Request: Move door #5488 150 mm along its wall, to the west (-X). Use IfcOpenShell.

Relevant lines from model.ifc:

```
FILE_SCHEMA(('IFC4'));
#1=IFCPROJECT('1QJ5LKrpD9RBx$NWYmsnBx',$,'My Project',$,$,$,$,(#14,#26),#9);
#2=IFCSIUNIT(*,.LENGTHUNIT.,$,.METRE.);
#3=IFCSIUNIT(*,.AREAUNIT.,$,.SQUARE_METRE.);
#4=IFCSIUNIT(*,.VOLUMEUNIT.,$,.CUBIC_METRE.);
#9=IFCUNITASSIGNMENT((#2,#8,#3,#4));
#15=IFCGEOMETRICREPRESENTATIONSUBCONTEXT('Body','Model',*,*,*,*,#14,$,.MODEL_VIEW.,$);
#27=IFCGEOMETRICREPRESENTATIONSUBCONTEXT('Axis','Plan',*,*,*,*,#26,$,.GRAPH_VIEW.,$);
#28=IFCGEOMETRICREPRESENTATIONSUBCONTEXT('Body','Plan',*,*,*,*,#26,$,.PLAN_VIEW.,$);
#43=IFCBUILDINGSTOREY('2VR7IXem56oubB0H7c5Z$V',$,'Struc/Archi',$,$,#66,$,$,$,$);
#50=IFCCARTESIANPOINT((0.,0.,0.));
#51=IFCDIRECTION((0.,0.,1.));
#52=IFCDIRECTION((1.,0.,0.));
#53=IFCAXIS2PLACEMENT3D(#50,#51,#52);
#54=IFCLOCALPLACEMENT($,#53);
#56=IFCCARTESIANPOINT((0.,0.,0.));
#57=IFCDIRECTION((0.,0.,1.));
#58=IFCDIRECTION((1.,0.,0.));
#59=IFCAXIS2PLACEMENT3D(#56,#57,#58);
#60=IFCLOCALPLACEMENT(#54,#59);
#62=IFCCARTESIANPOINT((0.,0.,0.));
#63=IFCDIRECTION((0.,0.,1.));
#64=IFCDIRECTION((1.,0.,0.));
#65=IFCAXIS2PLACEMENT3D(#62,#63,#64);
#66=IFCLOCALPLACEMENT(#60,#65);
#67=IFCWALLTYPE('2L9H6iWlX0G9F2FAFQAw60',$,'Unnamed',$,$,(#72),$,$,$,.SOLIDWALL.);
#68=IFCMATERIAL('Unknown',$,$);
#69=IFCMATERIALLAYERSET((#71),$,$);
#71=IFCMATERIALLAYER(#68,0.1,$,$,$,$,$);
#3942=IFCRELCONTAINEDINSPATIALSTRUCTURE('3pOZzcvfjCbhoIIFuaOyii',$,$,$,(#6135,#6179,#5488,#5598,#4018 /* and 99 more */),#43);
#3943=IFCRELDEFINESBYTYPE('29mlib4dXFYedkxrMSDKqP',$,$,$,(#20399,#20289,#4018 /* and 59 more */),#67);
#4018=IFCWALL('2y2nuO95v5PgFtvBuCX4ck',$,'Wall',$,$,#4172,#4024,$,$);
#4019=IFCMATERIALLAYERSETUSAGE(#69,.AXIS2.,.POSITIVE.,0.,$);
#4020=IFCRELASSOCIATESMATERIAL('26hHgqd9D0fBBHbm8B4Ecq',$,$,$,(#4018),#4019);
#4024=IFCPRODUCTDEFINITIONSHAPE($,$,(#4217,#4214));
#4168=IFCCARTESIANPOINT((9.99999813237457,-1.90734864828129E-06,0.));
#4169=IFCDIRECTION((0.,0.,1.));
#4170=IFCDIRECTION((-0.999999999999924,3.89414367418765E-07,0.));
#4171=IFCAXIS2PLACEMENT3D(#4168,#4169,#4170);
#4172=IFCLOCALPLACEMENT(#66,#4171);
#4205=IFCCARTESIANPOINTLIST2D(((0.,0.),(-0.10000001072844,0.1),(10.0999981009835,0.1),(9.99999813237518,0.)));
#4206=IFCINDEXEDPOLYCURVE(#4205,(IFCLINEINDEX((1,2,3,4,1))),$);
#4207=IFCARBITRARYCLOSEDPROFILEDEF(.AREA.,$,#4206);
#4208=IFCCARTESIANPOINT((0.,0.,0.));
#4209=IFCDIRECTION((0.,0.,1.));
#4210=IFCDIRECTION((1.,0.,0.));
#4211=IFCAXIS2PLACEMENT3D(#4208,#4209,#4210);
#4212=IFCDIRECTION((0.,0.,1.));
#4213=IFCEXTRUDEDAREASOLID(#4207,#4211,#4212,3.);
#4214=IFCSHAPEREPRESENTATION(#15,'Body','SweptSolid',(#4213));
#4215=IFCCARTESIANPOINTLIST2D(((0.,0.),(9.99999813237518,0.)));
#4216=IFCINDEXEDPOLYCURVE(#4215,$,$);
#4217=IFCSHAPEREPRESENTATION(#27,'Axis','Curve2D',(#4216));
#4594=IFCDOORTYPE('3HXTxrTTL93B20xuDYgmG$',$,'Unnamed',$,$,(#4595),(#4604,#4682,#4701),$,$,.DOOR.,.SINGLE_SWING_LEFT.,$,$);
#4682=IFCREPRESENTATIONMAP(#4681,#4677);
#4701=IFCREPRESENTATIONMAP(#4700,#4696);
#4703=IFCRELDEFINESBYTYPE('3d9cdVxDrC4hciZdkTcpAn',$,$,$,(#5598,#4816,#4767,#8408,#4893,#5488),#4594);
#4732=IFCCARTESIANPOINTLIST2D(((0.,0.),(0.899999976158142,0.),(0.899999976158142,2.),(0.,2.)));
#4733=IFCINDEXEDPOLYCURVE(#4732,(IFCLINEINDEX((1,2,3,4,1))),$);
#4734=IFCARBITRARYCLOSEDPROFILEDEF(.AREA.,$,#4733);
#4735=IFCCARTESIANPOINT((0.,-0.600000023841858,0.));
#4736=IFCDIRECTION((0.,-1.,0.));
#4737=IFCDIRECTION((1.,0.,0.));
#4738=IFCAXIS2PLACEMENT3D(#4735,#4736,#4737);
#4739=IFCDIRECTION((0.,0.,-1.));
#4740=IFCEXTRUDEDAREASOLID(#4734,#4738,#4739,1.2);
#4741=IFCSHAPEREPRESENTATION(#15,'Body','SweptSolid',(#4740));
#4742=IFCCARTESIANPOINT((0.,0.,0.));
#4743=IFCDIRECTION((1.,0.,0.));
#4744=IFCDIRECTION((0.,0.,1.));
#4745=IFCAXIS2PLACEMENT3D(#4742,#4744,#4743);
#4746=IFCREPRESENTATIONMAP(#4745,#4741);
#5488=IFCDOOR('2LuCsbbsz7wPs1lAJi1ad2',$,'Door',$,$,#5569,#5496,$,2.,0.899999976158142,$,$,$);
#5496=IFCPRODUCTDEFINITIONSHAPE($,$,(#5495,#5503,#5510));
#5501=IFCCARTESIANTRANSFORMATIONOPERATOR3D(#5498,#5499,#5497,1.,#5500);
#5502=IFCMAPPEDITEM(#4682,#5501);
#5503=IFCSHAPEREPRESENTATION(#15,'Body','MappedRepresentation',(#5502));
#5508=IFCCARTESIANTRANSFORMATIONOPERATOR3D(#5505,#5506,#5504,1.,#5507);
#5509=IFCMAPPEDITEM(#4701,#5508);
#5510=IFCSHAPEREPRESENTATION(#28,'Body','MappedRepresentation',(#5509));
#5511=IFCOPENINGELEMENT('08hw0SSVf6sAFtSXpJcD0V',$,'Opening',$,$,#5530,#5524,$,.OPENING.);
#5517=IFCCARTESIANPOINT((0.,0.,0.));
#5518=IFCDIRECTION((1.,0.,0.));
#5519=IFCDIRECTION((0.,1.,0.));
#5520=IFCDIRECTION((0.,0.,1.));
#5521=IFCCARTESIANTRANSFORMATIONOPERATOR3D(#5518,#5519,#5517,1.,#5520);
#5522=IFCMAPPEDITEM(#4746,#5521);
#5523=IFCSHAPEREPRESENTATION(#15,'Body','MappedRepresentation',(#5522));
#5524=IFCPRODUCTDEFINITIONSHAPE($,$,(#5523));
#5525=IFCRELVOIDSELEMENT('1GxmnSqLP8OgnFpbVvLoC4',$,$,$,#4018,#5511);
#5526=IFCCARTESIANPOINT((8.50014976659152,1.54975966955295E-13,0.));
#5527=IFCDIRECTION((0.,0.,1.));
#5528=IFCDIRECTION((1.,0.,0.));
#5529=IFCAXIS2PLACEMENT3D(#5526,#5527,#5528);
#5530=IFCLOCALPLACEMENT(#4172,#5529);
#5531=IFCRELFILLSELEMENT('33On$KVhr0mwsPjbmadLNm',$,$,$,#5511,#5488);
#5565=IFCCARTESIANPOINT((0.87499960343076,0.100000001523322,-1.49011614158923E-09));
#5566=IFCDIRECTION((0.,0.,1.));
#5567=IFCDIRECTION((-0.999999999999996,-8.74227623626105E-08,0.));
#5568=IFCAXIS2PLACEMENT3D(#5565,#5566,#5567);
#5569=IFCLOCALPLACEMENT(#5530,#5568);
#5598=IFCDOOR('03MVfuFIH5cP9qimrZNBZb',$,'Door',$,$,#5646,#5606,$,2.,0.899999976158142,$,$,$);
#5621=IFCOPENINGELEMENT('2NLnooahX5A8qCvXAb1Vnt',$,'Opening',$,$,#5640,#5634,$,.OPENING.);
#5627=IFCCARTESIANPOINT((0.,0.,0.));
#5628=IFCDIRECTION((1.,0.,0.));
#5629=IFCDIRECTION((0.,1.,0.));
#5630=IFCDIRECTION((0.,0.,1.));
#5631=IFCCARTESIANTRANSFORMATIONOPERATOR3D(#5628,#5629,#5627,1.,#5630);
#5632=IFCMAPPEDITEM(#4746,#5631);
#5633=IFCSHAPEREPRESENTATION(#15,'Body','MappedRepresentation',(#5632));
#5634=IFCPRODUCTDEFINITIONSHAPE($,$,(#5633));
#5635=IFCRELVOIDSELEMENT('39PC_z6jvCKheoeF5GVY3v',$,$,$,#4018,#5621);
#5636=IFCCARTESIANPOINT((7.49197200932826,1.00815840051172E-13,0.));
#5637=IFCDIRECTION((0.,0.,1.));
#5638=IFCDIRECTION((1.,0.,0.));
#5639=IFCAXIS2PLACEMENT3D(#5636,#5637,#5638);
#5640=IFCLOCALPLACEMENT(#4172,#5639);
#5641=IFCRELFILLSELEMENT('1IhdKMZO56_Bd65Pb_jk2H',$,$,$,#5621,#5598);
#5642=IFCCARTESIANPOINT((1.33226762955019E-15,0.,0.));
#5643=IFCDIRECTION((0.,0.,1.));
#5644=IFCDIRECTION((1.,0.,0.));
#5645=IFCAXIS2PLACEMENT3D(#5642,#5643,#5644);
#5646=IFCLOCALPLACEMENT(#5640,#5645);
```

```python
import ifcopenshell
import ifcopenshell.api.geometry
import ifcopenshell.util.placement
import ifcopenshell.util.unit

model = ifcopenshell.open("model.ifc")
unit_scale = ifcopenshell.util.unit.calculate_unit_scale(model)

door = model.by_guid("2LuCsbbsz7wPs1lAJi1ad2")
opening = door.FillsVoids[0].RelatingOpeningElement
wall = opening.VoidsElements[0].RelatingBuildingElement

wall_matrix = ifcopenshell.util.placement.get_local_placement(wall.ObjectPlacement)
shift = wall_matrix[:3, 0] * 0.15 / unit_scale
before = ifcopenshell.util.placement.get_local_placement(door.ObjectPlacement)[:3, 3].copy()

# The door is placed relative to its opening, so it follows when the opening moves.
matrix = ifcopenshell.util.placement.get_local_placement(opening.ObjectPlacement)
matrix[:3, 3] += shift
ifcopenshell.api.geometry.edit_object_placement(
    model, product=opening, matrix=matrix, is_si=False, should_transform_children=True
)

after = ifcopenshell.util.placement.get_local_placement(door.ObjectPlacement)[:3, 3]
print("door moved by", (after - before).round(3) + 0.0)

model.write("model_edited.ifc")
```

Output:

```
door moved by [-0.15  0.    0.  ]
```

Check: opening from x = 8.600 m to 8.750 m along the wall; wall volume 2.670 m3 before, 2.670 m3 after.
